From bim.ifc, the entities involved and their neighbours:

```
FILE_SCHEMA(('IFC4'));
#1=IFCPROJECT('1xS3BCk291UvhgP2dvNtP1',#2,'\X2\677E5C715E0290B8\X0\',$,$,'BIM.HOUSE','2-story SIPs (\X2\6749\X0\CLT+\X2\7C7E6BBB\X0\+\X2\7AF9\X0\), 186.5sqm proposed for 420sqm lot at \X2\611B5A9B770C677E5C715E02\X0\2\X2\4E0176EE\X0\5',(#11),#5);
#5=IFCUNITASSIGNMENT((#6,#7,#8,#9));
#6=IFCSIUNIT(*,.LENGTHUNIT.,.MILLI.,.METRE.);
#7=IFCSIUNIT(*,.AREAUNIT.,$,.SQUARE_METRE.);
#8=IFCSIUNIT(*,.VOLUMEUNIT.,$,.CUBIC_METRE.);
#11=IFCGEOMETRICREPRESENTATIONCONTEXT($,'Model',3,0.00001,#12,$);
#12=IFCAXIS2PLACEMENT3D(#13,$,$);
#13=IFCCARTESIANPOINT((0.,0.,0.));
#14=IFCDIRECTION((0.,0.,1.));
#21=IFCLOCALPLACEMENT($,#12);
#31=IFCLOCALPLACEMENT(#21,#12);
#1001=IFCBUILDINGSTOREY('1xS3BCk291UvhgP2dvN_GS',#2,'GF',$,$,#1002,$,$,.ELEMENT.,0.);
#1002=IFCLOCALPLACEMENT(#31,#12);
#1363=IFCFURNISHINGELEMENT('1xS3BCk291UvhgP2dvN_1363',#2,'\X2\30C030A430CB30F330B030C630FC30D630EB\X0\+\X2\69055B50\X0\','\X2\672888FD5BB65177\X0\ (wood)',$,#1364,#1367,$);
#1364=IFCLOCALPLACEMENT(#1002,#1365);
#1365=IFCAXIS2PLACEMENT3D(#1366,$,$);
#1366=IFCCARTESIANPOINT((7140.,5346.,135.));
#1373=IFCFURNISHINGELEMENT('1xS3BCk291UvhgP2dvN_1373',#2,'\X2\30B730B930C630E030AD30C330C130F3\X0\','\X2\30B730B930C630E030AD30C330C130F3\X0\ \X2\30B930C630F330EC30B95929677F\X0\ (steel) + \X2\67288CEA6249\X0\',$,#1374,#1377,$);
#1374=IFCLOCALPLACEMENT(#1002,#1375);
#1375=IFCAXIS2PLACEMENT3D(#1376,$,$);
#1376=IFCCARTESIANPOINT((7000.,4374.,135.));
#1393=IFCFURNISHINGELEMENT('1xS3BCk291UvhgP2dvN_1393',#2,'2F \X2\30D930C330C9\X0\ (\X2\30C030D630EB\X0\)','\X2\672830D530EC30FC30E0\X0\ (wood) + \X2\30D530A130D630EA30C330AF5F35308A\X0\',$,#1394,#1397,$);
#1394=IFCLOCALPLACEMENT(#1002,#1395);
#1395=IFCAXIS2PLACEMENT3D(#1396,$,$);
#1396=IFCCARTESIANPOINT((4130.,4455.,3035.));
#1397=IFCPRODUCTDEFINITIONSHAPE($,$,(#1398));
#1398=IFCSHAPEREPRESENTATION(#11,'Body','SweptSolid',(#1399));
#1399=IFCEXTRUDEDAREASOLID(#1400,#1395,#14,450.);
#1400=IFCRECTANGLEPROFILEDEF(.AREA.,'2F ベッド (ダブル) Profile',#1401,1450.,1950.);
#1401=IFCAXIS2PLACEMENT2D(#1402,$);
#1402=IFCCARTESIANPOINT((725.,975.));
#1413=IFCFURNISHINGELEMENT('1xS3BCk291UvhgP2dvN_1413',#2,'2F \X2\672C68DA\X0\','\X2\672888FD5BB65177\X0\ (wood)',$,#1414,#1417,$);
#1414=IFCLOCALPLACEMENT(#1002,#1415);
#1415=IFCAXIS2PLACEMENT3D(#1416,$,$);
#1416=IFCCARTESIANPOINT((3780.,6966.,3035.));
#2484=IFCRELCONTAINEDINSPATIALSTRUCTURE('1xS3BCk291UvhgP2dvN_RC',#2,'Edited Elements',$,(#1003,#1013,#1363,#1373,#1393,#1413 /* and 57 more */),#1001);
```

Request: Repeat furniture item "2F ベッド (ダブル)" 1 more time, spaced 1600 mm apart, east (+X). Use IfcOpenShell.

```python
import numpy as np
import ifcopenshell
import ifcopenshell.api.geometry
import ifcopenshell.api.root
import ifcopenshell.util.element
import ifcopenshell.util.placement
import ifcopenshell.util.unit

model = ifcopenshell.open("bim.ifc")
unit_scale = ifcopenshell.util.unit.calculate_unit_scale(model)


def reuse_history(source, copy):
    """copy_class also copies each property set's owner history, people and application; keep the originals."""
    for rel in copy.IsDefinedBy:
        if rel.is_a("IfcRelDefinesByProperties") and (history := rel.RelatingPropertyDefinition.OwnerHistory):
            rel.RelatingPropertyDefinition.OwnerHistory = source.OwnerHistory
            ifcopenshell.util.element.remove_deep2(model, history)


source = model.by_id(1393)
base = ifcopenshell.util.placement.get_local_placement(source.ObjectPlacement)
step = np.array([1.0, 0.0, 0.0]) * 1.6 / unit_scale

for i in range(1, 2):
    copy = ifcopenshell.api.root.copy_class(model, product=source)
    copy.Representation = ifcopenshell.util.element.copy_deep(
        model, source.Representation, exclude=["IfcGeometricRepresentationContext", "IfcRepresentationMap"]
    )
    reuse_history(source, copy)
    matrix = base.copy()
    matrix[:3, 3] += i * step
    print("added at", matrix[:3, 3].round(3) + 0.0)
    ifcopenshell.api.geometry.edit_object_placement(model, product=copy, matrix=matrix, is_si=False)

model.write("bim_updated.ifc")
```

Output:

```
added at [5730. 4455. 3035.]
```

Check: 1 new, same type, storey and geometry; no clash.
